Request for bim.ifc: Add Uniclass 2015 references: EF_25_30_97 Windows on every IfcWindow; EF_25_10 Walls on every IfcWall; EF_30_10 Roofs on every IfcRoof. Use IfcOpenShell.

First a look at what the model holds.

```python
import ifcopenshell

model = ifcopenshell.open("bim.ifc")
print(model.schema)
print("classifications:", [c.Name for c in model.by_type("IfcClassification")])
for ifc_class in ("IfcDoor", "IfcRoof", "IfcStair", "IfcWall", "IfcWindow"):
    print(ifc_class, len(model.by_type(ifc_class)))
```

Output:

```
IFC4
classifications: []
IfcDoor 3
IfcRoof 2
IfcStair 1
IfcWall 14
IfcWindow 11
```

```python
import ifcopenshell
import ifcopenshell.api.classification

model = ifcopenshell.open("bim.ifc")

system = ifcopenshell.api.classification.add_classification(model, classification="Uniclass 2015")

codes = {
    "IfcWindow": ("EF_25_30_97", "Windows"),
    "IfcWall": ("EF_25_10", "Walls"),
    "IfcRoof": ("EF_30_10", "Roofs"),
}
for ifc_class, (code, name) in codes.items():
    products = model.by_type(ifc_class)
    ifcopenshell.api.classification.add_reference(
        model, products=products, classification=system, identification=code, name=name
    )
    print(code, len(products))

model.write("bim_rev.ifc")
```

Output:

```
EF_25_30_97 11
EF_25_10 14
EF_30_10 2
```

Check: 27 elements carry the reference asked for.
